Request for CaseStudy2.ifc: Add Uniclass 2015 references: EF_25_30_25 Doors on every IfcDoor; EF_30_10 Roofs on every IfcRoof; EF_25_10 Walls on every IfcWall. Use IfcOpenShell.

First a look at what the model holds.

```python
import ifcopenshell

model = ifcopenshell.open("CaseStudy2.ifc")
print(model.schema)
print("classifications:", [c.Name for c in model.by_type("IfcClassification")])
for ifc_class in ("IfcDoor", "IfcRoof", "IfcStair", "IfcWall", "IfcWindow"):
    print(ifc_class, len(model.by_type(ifc_class)))
```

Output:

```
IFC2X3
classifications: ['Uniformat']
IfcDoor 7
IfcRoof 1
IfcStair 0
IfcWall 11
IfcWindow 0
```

```python
import ifcopenshell
import ifcopenshell.api.classification

model = ifcopenshell.open("CaseStudy2.ifc")

# IFC2X3 requires Source and Edition and has no link from the project to the system.
system = model.create_entity("IfcClassification", Source="NBS", Edition="2015", Name="Uniclass 2015")

codes = {
    "IfcDoor": ("EF_25_30_25", "Doors"),
    "IfcRoof": ("EF_30_10", "Roofs"),
    "IfcWall": ("EF_25_10", "Walls"),
}
for ifc_class, (code, name) in codes.items():
    products = model.by_type(ifc_class)
    ifcopenshell.api.classification.add_reference(
        model, products=products, classification=system, identification=code, name=name
    )
    print(code, len(products))

model.write("CaseStudy2_edited.ifc")
```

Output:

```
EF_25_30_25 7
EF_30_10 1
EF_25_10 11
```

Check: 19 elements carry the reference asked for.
